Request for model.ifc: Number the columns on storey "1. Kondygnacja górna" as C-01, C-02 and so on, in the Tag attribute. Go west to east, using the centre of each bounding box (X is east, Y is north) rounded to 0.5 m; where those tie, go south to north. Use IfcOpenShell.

First a look at what the model holds.

```python
import ifcopenshell
import ifcopenshell.util.element
import ifcopenshell.util.placement

model = ifcopenshell.open("model.ifc")
print(model.schema)
storey = next(s for s in model.by_type("IfcBuildingStorey") if s.Name == "1. Kondygnacja górna")
columns = [e for e in ifcopenshell.util.element.get_decomposition(storey) if e.is_a("IfcColumn")]
for e in sorted(columns, key=lambda e: e.id()):
    origin = ifcopenshell.util.placement.get_local_placement(e.ObjectPlacement)[:3, 3]
    print(e.id(), e.Tag, e.Name, origin.round(2) + 0.0, sep=" | ")
```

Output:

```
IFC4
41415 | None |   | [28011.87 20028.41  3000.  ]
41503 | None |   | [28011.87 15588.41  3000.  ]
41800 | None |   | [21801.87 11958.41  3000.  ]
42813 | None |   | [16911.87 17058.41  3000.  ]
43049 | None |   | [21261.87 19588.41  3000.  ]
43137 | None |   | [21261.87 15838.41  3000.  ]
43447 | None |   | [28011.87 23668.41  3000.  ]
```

```python
import ifcopenshell
import ifcopenshell.geom
import ifcopenshell.util.element
import ifcopenshell.util.shape

model = ifcopenshell.open("model.ifc")
settings = ifcopenshell.geom.settings()
settings.set("use-world-coords", True)


def centre(element):
    shape = ifcopenshell.geom.create_shape(settings, element)
    return ifcopenshell.util.shape.get_bbox_centroid(shape.geometry)


storey = next(s for s in model.by_type("IfcBuildingStorey") if s.Name == "1. Kondygnacja górna")
columns = [e for e in ifcopenshell.util.element.get_decomposition(storey) if e.is_a("IfcColumn")]

# Insertion points can sit at a corner or the storey origin, so sort by the geometry (in metres).
centres = {e: centre(e) for e in columns}
columns.sort(key=lambda e: (round(centres[e][0] / 0.5), centres[e][1]))

for i, e in enumerate(columns, start=1):
    number = f"C-{i:02d}"
    e.Tag = number
    print(e.id(), number)

model.write("model_rev.ifc")
```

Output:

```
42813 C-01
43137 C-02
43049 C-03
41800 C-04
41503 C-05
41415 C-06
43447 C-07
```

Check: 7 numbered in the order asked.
